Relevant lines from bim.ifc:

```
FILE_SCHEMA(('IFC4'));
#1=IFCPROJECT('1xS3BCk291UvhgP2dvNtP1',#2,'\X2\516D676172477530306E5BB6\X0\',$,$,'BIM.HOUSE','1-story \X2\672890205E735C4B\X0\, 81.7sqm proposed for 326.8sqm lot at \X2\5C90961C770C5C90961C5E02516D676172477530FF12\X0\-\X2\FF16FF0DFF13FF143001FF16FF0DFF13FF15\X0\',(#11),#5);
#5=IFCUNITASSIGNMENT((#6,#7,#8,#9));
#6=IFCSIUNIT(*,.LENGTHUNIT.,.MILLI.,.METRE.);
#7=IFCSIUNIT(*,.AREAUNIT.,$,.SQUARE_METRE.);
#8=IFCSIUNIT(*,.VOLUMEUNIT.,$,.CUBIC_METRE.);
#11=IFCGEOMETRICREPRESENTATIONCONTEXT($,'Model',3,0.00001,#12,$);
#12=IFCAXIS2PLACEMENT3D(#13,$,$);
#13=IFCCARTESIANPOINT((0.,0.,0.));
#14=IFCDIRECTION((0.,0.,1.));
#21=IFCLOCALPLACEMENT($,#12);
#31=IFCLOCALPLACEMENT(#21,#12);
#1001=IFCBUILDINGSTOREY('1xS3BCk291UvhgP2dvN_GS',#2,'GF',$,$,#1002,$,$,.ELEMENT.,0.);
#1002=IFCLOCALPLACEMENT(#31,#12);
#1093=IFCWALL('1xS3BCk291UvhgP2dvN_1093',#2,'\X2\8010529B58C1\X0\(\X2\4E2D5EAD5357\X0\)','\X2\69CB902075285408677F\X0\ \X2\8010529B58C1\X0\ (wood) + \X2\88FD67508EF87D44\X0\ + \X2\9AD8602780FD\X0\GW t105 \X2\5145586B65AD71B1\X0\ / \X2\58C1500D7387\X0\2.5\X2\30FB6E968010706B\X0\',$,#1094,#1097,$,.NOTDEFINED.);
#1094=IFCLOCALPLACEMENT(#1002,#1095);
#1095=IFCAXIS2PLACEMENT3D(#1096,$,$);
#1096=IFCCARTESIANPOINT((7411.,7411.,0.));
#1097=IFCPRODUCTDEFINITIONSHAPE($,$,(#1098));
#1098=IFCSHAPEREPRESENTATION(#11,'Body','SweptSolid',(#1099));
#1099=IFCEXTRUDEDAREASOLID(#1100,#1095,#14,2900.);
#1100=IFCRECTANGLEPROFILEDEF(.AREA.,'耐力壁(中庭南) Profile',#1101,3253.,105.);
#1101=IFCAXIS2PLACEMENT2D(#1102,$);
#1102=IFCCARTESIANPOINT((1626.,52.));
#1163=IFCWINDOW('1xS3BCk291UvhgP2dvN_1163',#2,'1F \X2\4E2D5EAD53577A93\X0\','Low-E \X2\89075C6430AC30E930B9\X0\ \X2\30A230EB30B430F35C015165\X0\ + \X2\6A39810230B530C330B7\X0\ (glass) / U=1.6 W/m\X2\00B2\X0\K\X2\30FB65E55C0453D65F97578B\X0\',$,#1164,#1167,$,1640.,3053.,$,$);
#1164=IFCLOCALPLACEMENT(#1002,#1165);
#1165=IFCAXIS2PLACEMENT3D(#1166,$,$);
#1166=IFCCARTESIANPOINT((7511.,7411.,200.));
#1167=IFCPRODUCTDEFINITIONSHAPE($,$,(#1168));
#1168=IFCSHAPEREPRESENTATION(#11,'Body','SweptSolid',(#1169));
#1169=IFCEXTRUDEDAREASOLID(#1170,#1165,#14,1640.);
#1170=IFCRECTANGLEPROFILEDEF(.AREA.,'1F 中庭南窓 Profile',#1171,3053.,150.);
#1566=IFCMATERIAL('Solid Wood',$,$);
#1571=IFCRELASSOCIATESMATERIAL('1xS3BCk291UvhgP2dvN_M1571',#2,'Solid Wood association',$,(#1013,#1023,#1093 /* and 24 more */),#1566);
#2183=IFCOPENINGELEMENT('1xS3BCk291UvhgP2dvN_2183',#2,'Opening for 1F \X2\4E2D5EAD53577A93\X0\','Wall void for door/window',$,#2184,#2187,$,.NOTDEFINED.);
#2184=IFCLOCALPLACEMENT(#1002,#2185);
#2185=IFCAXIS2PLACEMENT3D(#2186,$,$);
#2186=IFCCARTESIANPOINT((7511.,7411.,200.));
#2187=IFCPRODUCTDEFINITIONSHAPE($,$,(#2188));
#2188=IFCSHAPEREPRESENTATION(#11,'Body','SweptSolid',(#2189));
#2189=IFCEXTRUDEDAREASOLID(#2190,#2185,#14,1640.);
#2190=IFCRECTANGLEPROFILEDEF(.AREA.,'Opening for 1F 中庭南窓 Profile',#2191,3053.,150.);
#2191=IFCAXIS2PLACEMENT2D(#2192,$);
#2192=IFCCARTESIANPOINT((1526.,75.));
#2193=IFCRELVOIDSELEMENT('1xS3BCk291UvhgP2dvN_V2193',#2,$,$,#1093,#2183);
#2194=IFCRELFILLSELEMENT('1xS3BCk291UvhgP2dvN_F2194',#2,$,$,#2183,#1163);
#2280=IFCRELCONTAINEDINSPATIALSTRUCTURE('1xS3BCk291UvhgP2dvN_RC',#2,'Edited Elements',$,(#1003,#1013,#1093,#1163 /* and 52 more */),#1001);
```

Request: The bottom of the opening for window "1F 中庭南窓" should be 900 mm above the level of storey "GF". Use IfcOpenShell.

```python
import numpy as np
import ifcopenshell
import ifcopenshell.api.geometry
import ifcopenshell.geom
import ifcopenshell.util.element
import ifcopenshell.util.placement
import ifcopenshell.util.shape
import ifcopenshell.util.unit

model = ifcopenshell.open("bim.ifc")
unit_scale = ifcopenshell.util.unit.calculate_unit_scale(model)

window = model.by_guid("1xS3BCk291UvhgP2dvN_1163")
opening = window.FillsVoids[0].RelatingOpeningElement
storey = ifcopenshell.util.element.get_container(window, ifc_class="IfcBuildingStorey")
level = ifcopenshell.util.placement.get_local_placement(storey.ObjectPlacement)[2, 3]

# The opening's origin need not be at the sill, so measure its lowest point.
shape = ifcopenshell.geom.create_shape(ifcopenshell.geom.settings(), opening)
bottom = ifcopenshell.util.shape.get_shape_bottom_elevation(shape, shape.geometry) / unit_scale
dz = level + 0.9 / unit_scale - bottom

shift = np.array([0.0, 0.0, dz])
# The window is not placed relative to its opening, so move both.
for product in (opening, window):
    matrix = ifcopenshell.util.placement.get_local_placement(product.ObjectPlacement)
    matrix[:3, 3] += shift
    ifcopenshell.api.geometry.edit_object_placement(model, product=product, matrix=matrix, is_si=False)

print(f"moved by {dz * unit_scale:+.3f} m")

model.write("bim_v2.ifc")
```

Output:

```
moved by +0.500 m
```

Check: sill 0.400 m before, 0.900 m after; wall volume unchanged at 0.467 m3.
